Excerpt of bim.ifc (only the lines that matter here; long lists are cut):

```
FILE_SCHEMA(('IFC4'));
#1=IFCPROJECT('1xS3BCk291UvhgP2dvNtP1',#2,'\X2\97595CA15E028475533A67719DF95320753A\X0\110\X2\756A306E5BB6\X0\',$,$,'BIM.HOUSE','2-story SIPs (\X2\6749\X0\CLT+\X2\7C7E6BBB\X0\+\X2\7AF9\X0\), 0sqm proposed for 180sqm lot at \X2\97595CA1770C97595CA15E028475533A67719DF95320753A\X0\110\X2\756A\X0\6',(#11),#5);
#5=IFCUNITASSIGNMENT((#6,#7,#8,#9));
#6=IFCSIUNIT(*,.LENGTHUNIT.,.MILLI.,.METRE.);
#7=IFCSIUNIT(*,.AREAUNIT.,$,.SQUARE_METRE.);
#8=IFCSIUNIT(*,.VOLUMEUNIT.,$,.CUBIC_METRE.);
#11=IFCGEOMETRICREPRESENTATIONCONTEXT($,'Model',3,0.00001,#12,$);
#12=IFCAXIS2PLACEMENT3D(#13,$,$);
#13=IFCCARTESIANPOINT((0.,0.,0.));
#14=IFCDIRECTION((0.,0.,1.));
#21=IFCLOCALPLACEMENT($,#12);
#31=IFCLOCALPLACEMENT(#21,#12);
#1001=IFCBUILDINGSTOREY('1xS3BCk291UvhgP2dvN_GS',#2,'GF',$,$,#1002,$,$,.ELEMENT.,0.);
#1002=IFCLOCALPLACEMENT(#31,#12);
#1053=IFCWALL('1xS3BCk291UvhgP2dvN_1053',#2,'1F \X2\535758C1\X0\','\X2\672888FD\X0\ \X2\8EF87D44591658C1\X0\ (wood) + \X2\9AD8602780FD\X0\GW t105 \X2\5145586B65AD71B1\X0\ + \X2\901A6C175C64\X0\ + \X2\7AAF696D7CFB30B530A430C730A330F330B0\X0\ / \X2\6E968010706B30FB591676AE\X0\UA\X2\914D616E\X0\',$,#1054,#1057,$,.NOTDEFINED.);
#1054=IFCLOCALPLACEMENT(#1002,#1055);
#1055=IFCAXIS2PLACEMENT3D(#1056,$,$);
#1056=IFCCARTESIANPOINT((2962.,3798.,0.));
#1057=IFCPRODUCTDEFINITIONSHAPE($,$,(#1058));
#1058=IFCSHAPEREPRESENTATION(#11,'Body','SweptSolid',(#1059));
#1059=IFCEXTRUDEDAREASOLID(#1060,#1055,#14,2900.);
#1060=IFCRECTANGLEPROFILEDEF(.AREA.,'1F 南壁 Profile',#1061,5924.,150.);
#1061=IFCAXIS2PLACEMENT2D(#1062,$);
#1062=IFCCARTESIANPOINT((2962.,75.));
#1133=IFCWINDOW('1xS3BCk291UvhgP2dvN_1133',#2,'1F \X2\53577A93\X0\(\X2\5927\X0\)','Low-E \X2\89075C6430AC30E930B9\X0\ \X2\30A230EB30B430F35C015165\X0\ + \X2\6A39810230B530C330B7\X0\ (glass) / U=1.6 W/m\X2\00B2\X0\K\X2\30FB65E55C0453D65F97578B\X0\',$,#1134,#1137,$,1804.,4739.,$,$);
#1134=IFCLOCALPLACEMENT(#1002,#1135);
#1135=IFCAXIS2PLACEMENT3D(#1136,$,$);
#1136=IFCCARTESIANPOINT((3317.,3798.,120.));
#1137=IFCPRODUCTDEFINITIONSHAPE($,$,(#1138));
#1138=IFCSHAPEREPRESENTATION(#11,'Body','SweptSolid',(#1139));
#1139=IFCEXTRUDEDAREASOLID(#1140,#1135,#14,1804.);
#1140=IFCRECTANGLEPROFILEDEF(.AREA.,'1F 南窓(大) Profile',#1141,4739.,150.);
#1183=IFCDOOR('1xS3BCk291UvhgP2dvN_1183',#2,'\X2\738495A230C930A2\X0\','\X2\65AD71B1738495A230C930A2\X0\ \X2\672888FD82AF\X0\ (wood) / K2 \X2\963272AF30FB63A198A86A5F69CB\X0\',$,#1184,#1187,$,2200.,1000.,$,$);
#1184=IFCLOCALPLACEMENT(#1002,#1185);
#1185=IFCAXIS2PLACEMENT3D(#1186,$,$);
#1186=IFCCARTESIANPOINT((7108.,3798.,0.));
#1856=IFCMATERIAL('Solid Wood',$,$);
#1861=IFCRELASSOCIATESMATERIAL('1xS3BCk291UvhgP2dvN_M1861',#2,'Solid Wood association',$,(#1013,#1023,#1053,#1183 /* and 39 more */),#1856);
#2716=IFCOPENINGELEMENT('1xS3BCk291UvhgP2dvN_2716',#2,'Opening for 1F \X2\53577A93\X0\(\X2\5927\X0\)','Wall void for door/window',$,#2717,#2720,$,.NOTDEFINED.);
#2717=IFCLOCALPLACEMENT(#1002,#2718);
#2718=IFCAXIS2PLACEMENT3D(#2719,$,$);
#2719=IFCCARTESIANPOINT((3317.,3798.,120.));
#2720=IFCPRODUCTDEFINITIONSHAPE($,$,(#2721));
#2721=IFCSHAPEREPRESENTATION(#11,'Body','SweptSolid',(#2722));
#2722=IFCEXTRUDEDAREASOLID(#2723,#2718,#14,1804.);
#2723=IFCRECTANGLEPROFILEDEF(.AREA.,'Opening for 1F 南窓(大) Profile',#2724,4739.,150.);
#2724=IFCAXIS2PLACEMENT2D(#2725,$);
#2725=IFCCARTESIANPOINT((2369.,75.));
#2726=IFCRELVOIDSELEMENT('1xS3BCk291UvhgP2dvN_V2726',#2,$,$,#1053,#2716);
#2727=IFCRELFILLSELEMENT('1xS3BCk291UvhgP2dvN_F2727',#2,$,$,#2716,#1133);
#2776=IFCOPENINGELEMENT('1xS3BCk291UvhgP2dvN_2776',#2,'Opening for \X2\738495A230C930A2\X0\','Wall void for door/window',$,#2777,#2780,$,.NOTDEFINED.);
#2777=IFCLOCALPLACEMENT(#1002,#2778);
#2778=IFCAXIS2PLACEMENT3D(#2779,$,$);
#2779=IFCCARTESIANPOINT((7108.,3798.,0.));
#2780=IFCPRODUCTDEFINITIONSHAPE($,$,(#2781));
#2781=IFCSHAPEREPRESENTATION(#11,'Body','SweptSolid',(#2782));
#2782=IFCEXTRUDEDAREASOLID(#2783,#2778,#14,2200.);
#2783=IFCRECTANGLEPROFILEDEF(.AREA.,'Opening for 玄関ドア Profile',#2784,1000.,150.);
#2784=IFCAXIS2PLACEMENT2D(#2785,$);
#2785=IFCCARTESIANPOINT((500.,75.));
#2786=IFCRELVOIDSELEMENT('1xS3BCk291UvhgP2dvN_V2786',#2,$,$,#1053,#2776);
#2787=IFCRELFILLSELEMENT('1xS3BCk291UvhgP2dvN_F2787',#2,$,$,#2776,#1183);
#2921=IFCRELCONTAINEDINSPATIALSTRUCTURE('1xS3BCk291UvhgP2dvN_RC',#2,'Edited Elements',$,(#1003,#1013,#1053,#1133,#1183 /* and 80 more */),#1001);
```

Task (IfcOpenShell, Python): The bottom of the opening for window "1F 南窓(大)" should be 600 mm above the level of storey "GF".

```python
import numpy as np
import ifcopenshell
import ifcopenshell.api.geometry
import ifcopenshell.geom
import ifcopenshell.util.element
import ifcopenshell.util.placement
import ifcopenshell.util.shape
import ifcopenshell.util.unit

model = ifcopenshell.open("bim.ifc")
unit_scale = ifcopenshell.util.unit.calculate_unit_scale(model)

window = model.by_guid("1xS3BCk291UvhgP2dvN_1133")
opening = window.FillsVoids[0].RelatingOpeningElement
storey = ifcopenshell.util.element.get_container(window, ifc_class="IfcBuildingStorey")
level = ifcopenshell.util.placement.get_local_placement(storey.ObjectPlacement)[2, 3]

# The opening's origin need not be at the sill, so measure its lowest point.
shape = ifcopenshell.geom.create_shape(ifcopenshell.geom.settings(), opening)
bottom = ifcopenshell.util.shape.get_shape_bottom_elevation(shape, shape.geometry) / unit_scale
dz = level + 0.6 / unit_scale - bottom

shift = np.array([0.0, 0.0, dz])
# The window is not placed relative to its opening, so move both.
for product in (opening, window):
    matrix = ifcopenshell.util.placement.get_local_placement(product.ObjectPlacement)
    matrix[:3, 3] += shift
    ifcopenshell.api.geometry.edit_object_placement(model, product=product, matrix=matrix, is_si=False)

print(f"moved by {dz * unit_scale:+.3f} m")

model.write("bim-out.ifc")
```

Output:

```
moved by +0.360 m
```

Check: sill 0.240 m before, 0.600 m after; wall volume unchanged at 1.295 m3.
